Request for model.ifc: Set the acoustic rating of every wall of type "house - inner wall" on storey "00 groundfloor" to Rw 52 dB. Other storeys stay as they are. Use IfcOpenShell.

First a look at what the model holds.

```python
import ifcopenshell
import ifcopenshell.util.element

model = ifcopenshell.open("model.ifc")
print(model.schema)
storey = next(s for s in model.by_type("IfcBuildingStorey") if s.Name == "00 groundfloor")
walls = [e for e in ifcopenshell.util.element.get_decomposition(storey) if e.is_a("IfcWall")]
seen = {}
for e in walls:
    element_type = ifcopenshell.util.element.get_type(e)
    key = (element_type.Name if element_type != e and element_type else None, ifcopenshell.util.element.get_pset(e, "Pset_WallCommon", "AcousticRating"))
    seen[key] = seen.get(key, 0) + 1
for (name, value), count in sorted(seen.items(), key=str):
    print(count, "x", name, "|", value)
```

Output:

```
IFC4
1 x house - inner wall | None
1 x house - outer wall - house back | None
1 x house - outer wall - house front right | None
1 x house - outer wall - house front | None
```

```python
import ifcopenshell
import ifcopenshell.api.pset
import ifcopenshell.util.element

model = ifcopenshell.open("model.ifc")

storey = next(s for s in model.by_type("IfcBuildingStorey") if s.Name == "00 groundfloor")
walls = [e for e in ifcopenshell.util.element.get_decomposition(storey) if e.is_a("IfcWall")]

count = 0
for e in walls:
    element_type = ifcopenshell.util.element.get_type(e)
    if element_type in (None, e) or element_type.Name != "house - inner wall":
        continue
    # add_pset returns the element's existing set when there is one.
    pset = ifcopenshell.api.pset.add_pset(model, product=e, name="Pset_WallCommon")
    ifcopenshell.api.pset.edit_pset(model, pset=pset, properties={"AcousticRating": "Rw 52 dB"})
    count += 1

print(count, "walls updated")

model.write("model-out.ifc")
```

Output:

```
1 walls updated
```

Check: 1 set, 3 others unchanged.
